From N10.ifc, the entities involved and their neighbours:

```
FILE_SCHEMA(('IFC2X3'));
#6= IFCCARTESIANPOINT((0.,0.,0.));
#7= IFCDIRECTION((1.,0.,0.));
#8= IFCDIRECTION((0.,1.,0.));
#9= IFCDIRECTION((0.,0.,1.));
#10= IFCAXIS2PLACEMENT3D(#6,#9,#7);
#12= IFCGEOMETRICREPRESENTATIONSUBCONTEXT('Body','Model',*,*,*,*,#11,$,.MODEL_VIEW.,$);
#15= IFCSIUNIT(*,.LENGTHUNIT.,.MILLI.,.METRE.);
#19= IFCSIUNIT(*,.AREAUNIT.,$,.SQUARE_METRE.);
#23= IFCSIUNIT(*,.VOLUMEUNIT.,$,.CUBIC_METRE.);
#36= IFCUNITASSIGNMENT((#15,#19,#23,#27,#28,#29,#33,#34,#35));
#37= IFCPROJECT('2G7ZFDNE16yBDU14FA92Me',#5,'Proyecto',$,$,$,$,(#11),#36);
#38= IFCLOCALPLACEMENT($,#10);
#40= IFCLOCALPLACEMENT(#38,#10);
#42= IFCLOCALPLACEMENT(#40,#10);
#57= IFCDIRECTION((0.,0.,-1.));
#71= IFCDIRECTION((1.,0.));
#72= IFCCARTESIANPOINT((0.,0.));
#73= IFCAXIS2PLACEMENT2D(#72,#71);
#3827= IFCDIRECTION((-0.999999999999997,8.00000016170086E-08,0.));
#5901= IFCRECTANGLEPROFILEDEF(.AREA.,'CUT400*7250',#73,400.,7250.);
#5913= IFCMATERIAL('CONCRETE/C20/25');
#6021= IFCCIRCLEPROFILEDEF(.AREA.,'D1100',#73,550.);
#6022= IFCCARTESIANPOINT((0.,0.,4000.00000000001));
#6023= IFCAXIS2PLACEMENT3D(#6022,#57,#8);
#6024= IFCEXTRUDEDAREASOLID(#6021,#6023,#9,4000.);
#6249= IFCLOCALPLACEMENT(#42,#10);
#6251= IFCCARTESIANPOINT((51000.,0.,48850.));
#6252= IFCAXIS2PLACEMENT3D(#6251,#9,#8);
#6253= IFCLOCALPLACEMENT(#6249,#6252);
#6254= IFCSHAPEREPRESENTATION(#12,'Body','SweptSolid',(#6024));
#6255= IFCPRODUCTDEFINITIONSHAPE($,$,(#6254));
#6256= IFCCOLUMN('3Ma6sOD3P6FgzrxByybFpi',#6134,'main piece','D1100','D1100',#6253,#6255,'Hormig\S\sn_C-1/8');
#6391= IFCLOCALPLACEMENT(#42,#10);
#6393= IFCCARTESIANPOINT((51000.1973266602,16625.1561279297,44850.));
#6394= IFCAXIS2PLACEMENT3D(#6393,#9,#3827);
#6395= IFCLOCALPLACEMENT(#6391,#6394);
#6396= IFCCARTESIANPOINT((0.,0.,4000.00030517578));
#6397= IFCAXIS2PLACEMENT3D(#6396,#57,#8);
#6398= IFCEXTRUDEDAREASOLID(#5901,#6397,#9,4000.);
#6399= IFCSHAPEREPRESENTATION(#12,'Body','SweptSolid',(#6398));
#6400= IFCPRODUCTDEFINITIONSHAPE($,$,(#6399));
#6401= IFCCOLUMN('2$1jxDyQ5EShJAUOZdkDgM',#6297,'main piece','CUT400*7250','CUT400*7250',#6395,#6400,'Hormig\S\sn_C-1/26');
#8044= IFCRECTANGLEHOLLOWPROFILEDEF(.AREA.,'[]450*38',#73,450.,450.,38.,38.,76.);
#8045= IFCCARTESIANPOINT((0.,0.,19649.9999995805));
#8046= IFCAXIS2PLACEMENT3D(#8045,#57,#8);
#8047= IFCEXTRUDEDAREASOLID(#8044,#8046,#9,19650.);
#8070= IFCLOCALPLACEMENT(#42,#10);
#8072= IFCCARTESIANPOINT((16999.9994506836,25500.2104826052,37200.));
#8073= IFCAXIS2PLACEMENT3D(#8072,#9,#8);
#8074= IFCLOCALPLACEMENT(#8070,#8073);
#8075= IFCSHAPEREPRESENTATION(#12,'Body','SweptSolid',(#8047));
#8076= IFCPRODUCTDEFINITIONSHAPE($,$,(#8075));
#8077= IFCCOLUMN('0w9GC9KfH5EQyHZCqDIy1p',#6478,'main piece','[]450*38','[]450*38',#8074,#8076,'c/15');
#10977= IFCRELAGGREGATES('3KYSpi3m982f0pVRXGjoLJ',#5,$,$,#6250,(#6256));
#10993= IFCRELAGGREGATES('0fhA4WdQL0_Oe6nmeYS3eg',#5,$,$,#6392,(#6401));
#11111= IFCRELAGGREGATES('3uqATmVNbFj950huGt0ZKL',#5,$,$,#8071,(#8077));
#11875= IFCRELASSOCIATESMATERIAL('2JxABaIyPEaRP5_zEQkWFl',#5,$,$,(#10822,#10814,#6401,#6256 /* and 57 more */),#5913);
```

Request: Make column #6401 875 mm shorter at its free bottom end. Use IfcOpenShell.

```python
import ifcopenshell
import ifcopenshell.util.representation
import ifcopenshell.util.unit

model = ifcopenshell.open("N10.ifc")
unit_scale = ifcopenshell.util.unit.calculate_unit_scale(model)

member = model.by_guid("2$1jxDyQ5EShJAUOZdkDgM")
change = -0.875 / unit_scale

# The extrusion runs towards the end named, so only its depth changes.
body = ifcopenshell.util.representation.get_representation(member, "Model", "Body")
solid = body.Items[0]
old_length = solid.Depth
solid.Depth += change

print(f"length {old_length:g} -> {solid.Depth:g}")

model.write("N10_edited.ifc")
```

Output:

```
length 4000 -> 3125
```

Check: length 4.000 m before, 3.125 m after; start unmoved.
